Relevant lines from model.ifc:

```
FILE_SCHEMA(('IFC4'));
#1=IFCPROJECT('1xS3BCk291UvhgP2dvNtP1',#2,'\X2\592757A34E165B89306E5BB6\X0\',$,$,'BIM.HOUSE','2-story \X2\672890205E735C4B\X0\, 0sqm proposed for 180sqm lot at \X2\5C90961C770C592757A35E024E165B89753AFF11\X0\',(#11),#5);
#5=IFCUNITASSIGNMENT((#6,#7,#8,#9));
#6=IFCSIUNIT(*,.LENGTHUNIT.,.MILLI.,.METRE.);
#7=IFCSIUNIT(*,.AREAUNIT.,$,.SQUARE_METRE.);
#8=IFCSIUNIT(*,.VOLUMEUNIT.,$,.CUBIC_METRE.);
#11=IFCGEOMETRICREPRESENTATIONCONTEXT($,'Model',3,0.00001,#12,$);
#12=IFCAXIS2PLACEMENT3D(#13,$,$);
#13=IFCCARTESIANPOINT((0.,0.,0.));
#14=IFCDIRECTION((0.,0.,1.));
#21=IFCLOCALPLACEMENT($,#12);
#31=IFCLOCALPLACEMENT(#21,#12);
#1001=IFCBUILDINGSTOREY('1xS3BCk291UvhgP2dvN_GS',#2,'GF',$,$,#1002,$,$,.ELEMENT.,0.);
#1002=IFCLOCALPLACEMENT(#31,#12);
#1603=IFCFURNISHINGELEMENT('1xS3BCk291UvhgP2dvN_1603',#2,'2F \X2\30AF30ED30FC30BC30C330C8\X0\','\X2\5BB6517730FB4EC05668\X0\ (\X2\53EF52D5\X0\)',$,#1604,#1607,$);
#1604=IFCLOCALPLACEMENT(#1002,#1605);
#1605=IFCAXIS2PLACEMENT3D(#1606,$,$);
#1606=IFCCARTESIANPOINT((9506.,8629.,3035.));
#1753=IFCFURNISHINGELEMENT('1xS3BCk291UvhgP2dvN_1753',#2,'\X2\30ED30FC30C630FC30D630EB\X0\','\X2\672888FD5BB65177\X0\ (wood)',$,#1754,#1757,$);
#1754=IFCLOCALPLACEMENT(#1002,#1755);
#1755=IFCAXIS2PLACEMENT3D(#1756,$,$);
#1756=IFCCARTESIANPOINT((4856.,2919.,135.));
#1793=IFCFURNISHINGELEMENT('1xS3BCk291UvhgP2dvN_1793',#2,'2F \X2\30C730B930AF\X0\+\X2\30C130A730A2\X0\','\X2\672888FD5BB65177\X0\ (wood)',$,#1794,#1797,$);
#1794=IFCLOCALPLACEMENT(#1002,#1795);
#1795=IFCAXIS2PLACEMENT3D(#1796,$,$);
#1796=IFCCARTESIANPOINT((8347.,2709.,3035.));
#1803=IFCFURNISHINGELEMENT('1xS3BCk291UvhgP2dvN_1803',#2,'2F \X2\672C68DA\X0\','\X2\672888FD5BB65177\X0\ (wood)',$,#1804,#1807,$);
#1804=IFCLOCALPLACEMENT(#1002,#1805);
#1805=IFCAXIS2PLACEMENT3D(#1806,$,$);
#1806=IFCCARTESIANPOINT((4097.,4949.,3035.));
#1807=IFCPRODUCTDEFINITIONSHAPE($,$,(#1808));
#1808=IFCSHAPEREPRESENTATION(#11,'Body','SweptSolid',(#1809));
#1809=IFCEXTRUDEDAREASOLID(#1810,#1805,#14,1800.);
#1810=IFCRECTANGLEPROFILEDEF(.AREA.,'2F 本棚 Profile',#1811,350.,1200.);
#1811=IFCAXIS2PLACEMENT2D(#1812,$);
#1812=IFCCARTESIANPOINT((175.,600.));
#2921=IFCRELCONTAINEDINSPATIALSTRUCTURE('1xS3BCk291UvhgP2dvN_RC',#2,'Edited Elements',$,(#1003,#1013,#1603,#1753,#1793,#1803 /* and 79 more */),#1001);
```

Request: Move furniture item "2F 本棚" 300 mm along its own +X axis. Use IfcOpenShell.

```python
import ifcopenshell
import ifcopenshell.api.geometry
import ifcopenshell.util.placement

model = ifcopenshell.open("model.ifc")

item = model.by_id(1803)
matrix = ifcopenshell.util.placement.get_local_placement(item.ObjectPlacement)
matrix[:3, 3] += matrix[:3, 0] * 300.0
ifcopenshell.api.geometry.edit_object_placement(model, product=item, matrix=matrix, is_si=False)

print(ifcopenshell.util.placement.get_local_placement(item.ObjectPlacement).round(3) + 0.0)

model.write("model_updated.ifc")
```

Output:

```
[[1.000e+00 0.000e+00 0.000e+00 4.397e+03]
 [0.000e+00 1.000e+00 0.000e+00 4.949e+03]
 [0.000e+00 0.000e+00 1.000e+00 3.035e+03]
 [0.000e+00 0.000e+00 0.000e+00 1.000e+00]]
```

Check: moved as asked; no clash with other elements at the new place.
